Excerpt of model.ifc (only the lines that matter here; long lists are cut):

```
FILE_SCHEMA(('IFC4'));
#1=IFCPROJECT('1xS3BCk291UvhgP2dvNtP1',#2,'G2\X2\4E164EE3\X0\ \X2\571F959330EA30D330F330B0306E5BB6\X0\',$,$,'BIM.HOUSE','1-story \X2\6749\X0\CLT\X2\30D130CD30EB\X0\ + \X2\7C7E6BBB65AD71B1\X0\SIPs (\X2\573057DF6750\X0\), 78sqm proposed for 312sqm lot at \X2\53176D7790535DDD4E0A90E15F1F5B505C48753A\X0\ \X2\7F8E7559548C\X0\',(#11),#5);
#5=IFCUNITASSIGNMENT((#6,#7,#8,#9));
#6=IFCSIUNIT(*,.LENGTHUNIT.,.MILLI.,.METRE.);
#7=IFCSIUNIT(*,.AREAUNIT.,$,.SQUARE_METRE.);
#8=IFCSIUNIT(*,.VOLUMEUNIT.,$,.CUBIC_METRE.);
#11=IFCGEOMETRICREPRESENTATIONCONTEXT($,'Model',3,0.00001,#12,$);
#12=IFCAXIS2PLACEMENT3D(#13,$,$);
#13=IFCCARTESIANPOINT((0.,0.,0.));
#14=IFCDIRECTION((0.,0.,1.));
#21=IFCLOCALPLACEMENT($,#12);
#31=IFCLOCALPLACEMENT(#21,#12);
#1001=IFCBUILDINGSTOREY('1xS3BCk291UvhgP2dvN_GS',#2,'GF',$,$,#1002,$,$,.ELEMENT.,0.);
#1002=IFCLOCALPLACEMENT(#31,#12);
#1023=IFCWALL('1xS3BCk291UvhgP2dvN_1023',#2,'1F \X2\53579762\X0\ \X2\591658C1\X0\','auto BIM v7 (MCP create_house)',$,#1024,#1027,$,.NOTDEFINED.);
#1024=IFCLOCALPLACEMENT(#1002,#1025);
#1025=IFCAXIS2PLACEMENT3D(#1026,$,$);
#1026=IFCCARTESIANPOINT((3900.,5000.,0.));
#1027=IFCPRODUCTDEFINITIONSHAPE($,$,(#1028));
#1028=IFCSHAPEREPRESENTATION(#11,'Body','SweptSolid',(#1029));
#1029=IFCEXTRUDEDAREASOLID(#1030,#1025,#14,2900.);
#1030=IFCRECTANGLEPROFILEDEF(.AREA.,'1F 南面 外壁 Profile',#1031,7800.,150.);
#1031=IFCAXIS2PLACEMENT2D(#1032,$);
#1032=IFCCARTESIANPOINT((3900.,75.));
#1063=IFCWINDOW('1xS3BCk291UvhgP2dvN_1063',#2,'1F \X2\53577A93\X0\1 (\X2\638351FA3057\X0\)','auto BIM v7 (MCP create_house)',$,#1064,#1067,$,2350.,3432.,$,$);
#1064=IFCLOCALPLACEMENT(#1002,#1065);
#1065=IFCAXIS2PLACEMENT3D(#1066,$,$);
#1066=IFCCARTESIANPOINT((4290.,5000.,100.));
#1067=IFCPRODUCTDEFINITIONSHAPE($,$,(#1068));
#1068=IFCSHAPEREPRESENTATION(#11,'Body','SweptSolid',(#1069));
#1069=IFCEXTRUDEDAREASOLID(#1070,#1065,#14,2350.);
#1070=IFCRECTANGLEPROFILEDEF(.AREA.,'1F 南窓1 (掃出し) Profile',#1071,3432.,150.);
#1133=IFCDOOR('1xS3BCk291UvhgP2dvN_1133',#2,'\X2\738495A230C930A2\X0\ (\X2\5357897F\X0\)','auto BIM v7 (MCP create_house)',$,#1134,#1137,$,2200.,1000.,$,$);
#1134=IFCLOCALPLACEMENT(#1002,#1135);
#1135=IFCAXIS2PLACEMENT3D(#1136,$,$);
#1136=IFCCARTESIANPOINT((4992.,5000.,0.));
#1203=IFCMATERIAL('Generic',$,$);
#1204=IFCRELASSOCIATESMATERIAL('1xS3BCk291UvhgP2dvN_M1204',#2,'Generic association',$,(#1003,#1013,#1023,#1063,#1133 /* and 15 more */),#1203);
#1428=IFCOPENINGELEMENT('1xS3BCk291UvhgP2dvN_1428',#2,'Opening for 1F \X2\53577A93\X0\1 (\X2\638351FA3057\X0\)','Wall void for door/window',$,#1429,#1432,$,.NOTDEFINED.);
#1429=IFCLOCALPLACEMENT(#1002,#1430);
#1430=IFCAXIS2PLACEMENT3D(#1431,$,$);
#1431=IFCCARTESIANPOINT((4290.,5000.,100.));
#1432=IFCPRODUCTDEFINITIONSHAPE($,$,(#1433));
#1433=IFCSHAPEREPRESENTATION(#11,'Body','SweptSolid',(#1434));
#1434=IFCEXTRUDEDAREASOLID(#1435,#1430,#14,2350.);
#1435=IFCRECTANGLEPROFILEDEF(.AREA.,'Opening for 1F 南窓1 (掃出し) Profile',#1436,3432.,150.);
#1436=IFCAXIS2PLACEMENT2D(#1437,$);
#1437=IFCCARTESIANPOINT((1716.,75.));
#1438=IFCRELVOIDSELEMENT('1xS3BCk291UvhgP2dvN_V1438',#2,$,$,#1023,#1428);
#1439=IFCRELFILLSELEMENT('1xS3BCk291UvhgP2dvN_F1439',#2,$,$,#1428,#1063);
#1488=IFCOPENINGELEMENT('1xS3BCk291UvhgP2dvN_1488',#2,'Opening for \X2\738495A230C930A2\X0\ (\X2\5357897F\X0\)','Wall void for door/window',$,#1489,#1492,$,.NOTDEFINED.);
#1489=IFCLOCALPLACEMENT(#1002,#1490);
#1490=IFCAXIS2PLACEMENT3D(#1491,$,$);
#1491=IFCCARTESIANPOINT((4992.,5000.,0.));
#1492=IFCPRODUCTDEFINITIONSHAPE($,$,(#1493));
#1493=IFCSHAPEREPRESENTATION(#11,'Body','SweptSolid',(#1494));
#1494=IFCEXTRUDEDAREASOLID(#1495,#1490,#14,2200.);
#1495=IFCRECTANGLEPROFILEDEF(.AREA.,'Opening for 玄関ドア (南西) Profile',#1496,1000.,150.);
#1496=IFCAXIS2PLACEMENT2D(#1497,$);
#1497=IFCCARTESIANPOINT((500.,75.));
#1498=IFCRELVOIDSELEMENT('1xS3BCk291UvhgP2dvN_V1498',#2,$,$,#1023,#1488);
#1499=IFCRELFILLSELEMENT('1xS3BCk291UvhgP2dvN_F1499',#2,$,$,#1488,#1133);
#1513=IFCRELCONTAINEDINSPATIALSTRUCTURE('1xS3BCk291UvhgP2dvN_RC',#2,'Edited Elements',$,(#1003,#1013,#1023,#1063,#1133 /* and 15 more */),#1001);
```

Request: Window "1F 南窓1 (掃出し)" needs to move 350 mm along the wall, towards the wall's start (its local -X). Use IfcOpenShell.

```python
import ifcopenshell
import ifcopenshell.api.geometry
import ifcopenshell.util.placement

model = ifcopenshell.open("model.ifc")

window = model.by_guid("1xS3BCk291UvhgP2dvN_1063")
opening = window.FillsVoids[0].RelatingOpeningElement
wall = opening.VoidsElements[0].RelatingBuildingElement

wall_matrix = ifcopenshell.util.placement.get_local_placement(wall.ObjectPlacement)
shift = wall_matrix[:3, 0] * -350.0
before = ifcopenshell.util.placement.get_local_placement(window.ObjectPlacement)[:3, 3].copy()

# The window is not placed relative to its opening, so move both.
for product in (opening, window):
    matrix = ifcopenshell.util.placement.get_local_placement(product.ObjectPlacement)
    matrix[:3, 3] += shift
    ifcopenshell.api.geometry.edit_object_placement(model, product=product, matrix=matrix, is_si=False)

after = ifcopenshell.util.placement.get_local_placement(window.ObjectPlacement)[:3, 3]
print("window moved by", (after - before).round(3) + 0.0)

model.write("model-out.ifc")
```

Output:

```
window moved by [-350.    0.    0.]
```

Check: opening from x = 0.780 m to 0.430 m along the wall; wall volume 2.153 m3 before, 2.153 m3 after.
